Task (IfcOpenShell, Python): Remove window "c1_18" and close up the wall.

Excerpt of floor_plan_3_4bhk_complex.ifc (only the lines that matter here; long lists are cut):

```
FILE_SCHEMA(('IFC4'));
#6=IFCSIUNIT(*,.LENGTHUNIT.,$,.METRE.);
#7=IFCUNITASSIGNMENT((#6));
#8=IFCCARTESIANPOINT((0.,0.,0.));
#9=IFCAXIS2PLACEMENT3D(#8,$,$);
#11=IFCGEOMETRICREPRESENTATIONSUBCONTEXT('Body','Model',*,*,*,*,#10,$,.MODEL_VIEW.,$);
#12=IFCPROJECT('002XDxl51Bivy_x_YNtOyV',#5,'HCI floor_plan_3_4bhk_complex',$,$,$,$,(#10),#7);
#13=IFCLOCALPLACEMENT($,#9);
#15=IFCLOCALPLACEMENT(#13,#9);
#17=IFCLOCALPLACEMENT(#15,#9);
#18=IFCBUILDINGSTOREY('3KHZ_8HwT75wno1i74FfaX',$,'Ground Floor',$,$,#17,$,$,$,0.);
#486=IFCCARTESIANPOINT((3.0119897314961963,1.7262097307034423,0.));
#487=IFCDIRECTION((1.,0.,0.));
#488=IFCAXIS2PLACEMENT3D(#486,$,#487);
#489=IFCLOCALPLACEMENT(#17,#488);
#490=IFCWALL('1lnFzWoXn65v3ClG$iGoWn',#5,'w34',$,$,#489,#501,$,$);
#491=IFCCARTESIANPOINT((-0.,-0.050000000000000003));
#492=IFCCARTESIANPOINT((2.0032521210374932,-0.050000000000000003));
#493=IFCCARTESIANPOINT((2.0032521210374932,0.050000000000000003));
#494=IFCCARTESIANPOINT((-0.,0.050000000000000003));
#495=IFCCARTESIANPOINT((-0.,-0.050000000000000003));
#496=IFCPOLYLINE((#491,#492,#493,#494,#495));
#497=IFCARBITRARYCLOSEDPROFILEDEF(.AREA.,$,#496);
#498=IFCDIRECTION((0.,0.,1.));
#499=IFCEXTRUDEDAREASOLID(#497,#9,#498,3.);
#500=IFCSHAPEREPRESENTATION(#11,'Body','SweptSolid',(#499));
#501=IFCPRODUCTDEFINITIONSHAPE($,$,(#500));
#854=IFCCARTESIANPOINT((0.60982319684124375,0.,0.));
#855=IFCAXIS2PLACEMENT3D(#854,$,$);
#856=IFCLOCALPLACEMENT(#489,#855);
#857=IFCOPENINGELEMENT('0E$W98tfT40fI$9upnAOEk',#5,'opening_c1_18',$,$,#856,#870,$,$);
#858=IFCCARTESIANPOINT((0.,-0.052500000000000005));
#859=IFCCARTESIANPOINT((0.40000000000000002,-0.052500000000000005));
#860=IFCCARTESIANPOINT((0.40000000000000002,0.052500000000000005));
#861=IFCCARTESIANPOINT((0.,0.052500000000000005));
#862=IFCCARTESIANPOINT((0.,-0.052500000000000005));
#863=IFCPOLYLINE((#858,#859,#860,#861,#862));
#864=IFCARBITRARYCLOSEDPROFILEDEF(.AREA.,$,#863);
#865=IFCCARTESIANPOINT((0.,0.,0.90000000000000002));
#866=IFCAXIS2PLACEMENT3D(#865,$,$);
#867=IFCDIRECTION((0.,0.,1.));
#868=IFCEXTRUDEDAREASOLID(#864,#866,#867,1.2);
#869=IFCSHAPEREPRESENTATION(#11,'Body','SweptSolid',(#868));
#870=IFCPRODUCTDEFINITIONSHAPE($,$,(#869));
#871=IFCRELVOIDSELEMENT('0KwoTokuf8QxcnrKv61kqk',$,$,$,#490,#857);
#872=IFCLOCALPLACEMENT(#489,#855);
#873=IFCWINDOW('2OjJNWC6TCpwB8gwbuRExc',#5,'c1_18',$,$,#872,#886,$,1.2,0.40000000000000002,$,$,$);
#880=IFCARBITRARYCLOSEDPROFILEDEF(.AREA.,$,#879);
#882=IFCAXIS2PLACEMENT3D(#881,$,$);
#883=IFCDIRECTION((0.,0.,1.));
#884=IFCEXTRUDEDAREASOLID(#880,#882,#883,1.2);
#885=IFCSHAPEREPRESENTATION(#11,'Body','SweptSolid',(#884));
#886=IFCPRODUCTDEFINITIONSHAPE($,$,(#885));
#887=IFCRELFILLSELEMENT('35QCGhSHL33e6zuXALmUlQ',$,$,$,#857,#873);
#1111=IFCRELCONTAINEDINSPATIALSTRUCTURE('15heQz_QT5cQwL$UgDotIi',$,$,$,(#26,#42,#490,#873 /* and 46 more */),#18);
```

```python
import ifcopenshell
import ifcopenshell.api.feature
import ifcopenshell.api.root
import ifcopenshell.geom
import ifcopenshell.util.shape

model = ifcopenshell.open("floor_plan_3_4bhk_complex.ifc")
settings = ifcopenshell.geom.settings()


def volume(element):
    """Net volume in cubic metres, openings subtracted."""
    shape = ifcopenshell.geom.create_shape(settings, element)
    return ifcopenshell.util.shape.get_volume(shape.geometry)


window = model.by_id(873)
opening = window.FillsVoids[0].RelatingOpeningElement
wall = opening.VoidsElements[0].RelatingBuildingElement
before = volume(wall)

ifcopenshell.api.root.remove_product(model, product=window)
ifcopenshell.api.feature.remove_feature(model, feature=opening)

after = volume(wall)

print(f"wall volume {before:.3f} -> {after:.3f} m3")

model.write("floor_plan_3_4bhk_complex_rev.ifc")
```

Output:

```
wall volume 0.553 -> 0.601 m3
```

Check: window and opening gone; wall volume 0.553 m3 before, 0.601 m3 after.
